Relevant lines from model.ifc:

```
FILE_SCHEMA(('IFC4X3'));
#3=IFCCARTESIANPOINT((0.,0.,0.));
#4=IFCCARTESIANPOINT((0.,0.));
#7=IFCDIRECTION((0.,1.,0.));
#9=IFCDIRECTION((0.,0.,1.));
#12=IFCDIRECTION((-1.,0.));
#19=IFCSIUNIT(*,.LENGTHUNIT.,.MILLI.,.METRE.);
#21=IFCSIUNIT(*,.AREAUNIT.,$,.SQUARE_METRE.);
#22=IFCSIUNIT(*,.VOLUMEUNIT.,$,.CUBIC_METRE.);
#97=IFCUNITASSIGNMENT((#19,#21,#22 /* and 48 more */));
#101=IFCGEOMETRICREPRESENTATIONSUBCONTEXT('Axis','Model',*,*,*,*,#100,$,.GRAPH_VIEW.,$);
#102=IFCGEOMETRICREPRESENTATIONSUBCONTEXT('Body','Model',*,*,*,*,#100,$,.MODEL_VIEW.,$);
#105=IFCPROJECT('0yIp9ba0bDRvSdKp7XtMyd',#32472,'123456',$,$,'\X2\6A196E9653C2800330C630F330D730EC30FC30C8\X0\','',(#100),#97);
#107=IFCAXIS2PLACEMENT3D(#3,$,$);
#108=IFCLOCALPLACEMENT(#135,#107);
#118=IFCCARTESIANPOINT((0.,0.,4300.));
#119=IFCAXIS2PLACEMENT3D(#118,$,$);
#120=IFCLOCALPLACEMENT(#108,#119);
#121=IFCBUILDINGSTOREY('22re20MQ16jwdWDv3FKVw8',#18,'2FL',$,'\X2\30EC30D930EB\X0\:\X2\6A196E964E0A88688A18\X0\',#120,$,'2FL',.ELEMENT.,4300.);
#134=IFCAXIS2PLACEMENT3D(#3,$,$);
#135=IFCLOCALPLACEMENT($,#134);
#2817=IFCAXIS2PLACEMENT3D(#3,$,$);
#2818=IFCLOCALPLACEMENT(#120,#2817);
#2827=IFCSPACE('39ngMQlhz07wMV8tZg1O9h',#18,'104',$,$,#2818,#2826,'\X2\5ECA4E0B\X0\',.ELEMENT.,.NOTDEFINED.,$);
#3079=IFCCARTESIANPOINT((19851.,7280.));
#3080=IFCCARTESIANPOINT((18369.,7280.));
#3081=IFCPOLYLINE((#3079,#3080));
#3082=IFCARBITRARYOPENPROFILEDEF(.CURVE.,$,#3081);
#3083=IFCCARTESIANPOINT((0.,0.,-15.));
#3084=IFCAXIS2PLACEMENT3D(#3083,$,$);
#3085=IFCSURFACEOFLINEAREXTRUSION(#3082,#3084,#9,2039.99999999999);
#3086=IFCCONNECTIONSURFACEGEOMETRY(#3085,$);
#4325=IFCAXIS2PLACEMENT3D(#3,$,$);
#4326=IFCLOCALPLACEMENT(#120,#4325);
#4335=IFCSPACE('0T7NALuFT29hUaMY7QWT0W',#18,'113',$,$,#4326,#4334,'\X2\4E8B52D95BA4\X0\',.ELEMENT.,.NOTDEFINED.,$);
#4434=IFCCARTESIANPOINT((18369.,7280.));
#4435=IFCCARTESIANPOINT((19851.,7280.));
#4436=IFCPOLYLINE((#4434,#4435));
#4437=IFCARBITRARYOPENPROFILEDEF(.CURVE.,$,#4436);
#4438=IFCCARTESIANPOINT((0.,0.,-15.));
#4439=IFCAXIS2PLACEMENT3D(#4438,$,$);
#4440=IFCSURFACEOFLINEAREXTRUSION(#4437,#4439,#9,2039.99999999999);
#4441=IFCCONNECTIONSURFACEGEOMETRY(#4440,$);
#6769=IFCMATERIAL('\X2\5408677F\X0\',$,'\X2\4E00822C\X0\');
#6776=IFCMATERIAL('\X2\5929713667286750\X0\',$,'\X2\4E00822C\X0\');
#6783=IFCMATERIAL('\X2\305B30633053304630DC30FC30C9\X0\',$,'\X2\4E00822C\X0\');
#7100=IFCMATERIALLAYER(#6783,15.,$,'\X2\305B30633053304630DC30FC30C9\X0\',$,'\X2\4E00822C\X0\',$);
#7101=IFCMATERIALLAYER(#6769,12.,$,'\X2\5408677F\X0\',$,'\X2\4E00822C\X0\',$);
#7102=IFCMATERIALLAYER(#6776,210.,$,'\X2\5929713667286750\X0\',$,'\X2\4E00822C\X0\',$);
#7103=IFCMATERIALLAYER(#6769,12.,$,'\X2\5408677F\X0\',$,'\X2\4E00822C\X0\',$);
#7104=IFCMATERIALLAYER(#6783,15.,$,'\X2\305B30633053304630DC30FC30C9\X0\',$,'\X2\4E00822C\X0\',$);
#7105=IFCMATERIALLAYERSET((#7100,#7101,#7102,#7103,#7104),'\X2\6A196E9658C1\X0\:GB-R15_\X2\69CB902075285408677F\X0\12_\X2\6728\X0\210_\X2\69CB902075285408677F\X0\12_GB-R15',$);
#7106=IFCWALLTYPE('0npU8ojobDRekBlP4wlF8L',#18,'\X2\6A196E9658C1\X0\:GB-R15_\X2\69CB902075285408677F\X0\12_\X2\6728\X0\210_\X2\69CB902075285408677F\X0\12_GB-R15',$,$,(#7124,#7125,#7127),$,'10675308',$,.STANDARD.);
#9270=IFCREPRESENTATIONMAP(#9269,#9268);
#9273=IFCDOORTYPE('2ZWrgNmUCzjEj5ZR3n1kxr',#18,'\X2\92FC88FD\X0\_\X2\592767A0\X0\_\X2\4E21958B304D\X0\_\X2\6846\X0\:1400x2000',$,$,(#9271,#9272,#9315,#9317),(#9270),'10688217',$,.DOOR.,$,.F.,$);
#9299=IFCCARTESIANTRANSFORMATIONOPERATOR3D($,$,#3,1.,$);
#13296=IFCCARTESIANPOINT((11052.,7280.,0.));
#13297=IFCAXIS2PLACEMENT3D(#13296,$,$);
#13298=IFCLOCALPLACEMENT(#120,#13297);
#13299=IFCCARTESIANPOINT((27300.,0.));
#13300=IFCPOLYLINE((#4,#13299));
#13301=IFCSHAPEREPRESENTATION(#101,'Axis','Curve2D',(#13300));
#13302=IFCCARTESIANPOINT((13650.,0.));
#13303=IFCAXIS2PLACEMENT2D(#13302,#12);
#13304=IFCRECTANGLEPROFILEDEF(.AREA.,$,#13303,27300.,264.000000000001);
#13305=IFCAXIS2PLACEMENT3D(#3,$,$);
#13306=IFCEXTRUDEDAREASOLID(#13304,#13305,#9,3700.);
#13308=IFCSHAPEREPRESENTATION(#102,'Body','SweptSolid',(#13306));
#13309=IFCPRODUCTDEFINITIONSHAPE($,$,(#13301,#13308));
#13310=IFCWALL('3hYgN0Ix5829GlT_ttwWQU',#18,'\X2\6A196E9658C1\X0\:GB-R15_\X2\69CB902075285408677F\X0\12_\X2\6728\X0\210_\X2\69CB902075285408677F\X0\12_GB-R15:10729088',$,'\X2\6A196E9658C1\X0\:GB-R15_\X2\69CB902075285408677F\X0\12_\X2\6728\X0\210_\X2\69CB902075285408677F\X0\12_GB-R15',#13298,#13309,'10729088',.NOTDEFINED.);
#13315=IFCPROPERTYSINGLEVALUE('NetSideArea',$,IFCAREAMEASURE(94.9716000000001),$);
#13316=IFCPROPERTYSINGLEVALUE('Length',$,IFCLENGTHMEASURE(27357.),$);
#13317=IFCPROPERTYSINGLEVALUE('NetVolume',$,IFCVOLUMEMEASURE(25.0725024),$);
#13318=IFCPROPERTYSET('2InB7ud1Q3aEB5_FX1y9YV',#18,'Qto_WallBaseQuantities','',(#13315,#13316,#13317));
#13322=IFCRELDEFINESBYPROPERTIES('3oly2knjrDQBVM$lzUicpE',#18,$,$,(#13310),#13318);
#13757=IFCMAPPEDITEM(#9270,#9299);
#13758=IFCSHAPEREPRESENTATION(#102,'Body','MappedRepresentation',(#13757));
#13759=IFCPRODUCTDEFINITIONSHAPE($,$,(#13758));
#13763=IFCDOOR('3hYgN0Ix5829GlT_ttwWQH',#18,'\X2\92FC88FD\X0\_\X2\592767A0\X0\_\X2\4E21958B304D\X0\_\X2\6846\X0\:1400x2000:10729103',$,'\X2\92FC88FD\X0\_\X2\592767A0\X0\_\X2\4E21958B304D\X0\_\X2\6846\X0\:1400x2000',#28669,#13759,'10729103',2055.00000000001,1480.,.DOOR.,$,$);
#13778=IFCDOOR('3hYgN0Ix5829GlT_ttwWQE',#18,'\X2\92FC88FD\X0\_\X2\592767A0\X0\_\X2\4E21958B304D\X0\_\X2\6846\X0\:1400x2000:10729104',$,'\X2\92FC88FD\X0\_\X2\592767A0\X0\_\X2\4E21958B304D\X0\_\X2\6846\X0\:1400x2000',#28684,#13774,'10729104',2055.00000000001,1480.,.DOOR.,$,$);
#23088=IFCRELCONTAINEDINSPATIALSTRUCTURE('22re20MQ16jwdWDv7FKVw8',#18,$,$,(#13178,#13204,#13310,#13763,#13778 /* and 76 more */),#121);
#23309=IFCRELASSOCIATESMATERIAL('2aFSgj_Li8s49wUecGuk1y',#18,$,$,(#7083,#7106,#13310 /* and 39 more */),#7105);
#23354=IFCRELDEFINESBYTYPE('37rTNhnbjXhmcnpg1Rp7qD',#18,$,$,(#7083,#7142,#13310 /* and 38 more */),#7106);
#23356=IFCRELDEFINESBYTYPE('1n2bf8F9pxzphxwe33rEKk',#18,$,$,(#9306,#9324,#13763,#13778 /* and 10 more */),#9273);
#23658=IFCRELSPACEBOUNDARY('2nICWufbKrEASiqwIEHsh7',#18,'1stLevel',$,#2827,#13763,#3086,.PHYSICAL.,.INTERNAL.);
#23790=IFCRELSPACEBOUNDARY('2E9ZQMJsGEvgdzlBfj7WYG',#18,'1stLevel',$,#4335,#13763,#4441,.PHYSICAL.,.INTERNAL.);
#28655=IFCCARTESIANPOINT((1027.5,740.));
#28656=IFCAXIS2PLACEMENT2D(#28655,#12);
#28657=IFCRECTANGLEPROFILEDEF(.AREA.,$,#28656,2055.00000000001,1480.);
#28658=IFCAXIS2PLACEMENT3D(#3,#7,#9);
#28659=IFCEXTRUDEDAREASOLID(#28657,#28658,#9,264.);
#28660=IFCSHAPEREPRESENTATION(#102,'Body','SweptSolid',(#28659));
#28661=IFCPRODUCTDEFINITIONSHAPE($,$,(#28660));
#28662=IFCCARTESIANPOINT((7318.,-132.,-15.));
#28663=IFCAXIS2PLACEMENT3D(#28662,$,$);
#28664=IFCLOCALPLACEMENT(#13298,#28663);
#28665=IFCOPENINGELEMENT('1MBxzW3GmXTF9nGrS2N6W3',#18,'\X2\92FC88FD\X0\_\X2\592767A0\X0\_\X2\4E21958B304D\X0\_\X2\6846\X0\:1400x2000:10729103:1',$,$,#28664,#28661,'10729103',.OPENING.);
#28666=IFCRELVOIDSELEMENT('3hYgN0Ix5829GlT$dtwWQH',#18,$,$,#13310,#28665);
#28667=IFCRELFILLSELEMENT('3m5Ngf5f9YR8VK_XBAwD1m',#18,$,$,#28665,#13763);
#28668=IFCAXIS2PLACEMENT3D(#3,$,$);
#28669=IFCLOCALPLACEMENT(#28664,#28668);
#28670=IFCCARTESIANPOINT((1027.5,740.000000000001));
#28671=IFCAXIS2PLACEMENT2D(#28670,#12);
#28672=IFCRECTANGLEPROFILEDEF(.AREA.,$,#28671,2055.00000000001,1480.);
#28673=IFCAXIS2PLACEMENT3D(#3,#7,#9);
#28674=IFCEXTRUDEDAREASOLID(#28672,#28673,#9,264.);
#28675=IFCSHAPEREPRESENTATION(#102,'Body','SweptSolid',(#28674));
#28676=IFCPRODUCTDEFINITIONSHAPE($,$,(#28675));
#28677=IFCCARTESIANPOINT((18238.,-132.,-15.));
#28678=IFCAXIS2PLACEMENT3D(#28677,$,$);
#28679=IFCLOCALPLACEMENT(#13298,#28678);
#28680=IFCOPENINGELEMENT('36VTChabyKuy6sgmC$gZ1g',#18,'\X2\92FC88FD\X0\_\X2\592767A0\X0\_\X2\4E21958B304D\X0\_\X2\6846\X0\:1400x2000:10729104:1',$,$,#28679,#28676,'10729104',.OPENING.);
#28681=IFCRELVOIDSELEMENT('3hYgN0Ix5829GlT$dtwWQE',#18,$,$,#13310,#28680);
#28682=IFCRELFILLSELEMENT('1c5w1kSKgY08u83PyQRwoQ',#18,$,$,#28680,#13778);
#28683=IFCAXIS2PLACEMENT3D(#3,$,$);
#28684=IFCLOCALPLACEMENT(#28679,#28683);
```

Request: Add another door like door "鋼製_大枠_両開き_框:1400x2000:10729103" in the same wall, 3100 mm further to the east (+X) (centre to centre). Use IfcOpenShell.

```python
import numpy as np
import ifcopenshell
import ifcopenshell.api.feature
import ifcopenshell.api.geometry
import ifcopenshell.api.pset
import ifcopenshell.api.root
import ifcopenshell.geom
import ifcopenshell.util.element
import ifcopenshell.util.placement
import ifcopenshell.util.shape
import ifcopenshell.util.unit

model = ifcopenshell.open("model.ifc")
area_scale = ifcopenshell.util.unit.calculate_unit_scale(model, "AREAUNIT")
volume_scale = ifcopenshell.util.unit.calculate_unit_scale(model, "VOLUMEUNIT")
settings = ifcopenshell.geom.settings()


def volume(element):
    """Net volume in cubic metres, openings subtracted."""
    shape = ifcopenshell.geom.create_shape(settings, element)
    return ifcopenshell.util.shape.get_volume(shape.geometry)


def reuse_history(source, copy):
    """copy_class also copies each property set's owner history, people and application; keep the originals."""
    for rel in copy.IsDefinedBy:
        if rel.is_a("IfcRelDefinesByProperties") and (history := rel.RelatingPropertyDefinition.OwnerHistory):
            rel.RelatingPropertyDefinition.OwnerHistory = source.OwnerHistory
            ifcopenshell.util.element.remove_deep2(model, history)


door = model.by_guid("3hYgN0Ix5829GlT_ttwWQH")
opening = door.FillsVoids[0].RelatingOpeningElement
wall = opening.VoidsElements[0].RelatingBuildingElement
before = volume(wall)
shift = ifcopenshell.util.placement.get_local_placement(wall.ObjectPlacement)[:3, 0] * 3100.0

# copy_class copies the void relationship, type, container and properties, but no geometry.
new_opening = ifcopenshell.api.root.copy_class(model, product=opening)
new_opening.Representation = ifcopenshell.util.element.copy_deep(
    model, opening.Representation, exclude=["IfcGeometricRepresentationContext", "IfcRepresentationMap"]
)
new_opening.Name = "鋼製_大枠_両開き_框:1400x2000"
new_opening.Tag = None
new_door = ifcopenshell.api.root.copy_class(model, product=door)
new_door.Representation = ifcopenshell.util.element.copy_deep(
    model, door.Representation, exclude=["IfcGeometricRepresentationContext", "IfcRepresentationMap"]
)
new_door.Name = "鋼製_大枠_両開き_框:1400x2000"
new_door.Tag = None
reuse_history(door, new_door)
ifcopenshell.api.feature.add_filling(model, opening=new_opening, element=new_door)

for old, new in ((opening, new_opening), (door, new_door)):
    matrix = ifcopenshell.util.placement.get_local_placement(old.ObjectPlacement)
    matrix[:3, 3] += shift
    ifcopenshell.api.geometry.edit_object_placement(model, product=new, matrix=matrix, is_si=False)

# The copied space boundaries still share their surfaces with the original.
for rel in new_door.ProvidesBoundaries:
    if rel.ConnectionGeometry:
        rel.ConnectionGeometry = ifcopenshell.util.element.copy_deep(model, rel.ConnectionGeometry)

# Space boundary surfaces are stored in each space's coordinates; move them too.
for rel in new_door.ProvidesBoundaries:
    if not rel.ConnectionGeometry:
        continue
    surface = rel.ConnectionGeometry.SurfaceOnRelatingElement
    space_matrix = ifcopenshell.util.placement.get_local_placement(rel.RelatingSpace.ObjectPlacement)
    point = np.array(surface.Position.Location.Coordinates) + space_matrix[:3, :3].T @ shift
    surface.Position = model.createIfcAxis2Placement3D(
        model.createIfcCartesianPoint(point.tolist()), surface.Position.Axis, surface.Position.RefDirection
    )

after = volume(wall)
thickness = 0.264  # wall thickness in metres

# Update the wall's stored quantities.
pset = model.by_id(ifcopenshell.util.element.get_pset(wall, "Qto_WallBaseQuantities", should_inherit=False)["id"])
ifcopenshell.api.pset.edit_pset(model, pset=pset, properties={
    "NetSideArea": model.create_entity("IfcAreaMeasure", after / thickness / area_scale),
    "NetVolume": model.create_entity("IfcVolumeMeasure", after / volume_scale),
})

print(f"wall volume {before:.3f} -> {after:.3f} m3")

model.write("model-out.ifc")
```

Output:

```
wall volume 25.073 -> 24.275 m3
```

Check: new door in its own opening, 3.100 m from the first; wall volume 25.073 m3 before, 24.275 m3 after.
